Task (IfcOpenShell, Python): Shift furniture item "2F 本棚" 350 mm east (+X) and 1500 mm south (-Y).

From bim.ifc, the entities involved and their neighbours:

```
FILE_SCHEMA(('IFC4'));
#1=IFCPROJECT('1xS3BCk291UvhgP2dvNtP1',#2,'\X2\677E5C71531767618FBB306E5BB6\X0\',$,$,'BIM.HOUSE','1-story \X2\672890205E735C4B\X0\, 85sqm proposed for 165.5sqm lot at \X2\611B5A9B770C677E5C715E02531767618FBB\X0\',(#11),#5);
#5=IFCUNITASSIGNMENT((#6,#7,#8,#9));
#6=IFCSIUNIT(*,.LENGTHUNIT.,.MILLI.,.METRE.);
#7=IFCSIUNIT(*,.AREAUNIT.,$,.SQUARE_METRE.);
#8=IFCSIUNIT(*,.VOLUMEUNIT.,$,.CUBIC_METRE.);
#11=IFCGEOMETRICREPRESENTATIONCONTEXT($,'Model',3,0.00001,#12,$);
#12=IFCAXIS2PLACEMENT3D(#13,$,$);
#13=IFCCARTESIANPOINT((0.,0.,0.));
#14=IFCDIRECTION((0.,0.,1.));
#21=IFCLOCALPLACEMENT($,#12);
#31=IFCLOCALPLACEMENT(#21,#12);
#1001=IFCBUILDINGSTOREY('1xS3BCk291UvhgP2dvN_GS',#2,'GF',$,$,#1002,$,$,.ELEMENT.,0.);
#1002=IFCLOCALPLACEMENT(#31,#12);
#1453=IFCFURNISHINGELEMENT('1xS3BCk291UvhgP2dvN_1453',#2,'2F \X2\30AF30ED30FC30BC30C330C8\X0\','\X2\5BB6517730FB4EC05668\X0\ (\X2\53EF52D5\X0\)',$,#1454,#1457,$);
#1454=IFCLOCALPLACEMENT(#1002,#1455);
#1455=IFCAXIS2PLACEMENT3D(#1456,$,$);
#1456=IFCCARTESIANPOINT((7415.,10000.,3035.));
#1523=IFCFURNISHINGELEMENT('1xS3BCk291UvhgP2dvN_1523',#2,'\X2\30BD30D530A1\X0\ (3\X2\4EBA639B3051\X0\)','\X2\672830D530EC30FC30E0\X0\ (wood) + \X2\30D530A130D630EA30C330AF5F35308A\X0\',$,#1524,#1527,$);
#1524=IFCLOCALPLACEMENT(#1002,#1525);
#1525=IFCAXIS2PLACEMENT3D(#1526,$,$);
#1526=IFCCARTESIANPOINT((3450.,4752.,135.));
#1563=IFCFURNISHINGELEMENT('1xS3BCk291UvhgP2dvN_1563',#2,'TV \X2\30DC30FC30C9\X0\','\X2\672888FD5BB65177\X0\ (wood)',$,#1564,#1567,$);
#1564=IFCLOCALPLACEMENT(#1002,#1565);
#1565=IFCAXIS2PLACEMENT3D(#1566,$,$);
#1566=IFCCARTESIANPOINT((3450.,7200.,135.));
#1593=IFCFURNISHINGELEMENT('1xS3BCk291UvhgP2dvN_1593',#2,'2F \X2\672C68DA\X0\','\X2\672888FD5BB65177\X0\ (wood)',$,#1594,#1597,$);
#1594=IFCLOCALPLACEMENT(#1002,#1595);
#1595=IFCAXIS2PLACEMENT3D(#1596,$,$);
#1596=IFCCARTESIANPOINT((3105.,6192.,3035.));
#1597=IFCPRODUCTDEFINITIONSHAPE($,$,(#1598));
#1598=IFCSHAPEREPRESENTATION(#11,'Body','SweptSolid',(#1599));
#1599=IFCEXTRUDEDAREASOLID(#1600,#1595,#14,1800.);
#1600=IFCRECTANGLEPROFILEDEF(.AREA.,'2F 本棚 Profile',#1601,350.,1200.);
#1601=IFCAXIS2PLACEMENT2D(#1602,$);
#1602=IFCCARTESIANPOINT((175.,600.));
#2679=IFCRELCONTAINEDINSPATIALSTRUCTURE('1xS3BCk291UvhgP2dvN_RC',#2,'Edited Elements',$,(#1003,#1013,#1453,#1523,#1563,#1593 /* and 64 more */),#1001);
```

```python
import ifcopenshell
import ifcopenshell.api.geometry
import ifcopenshell.util.placement

model = ifcopenshell.open("bim.ifc")

item = model.by_guid("1xS3BCk291UvhgP2dvN_1593")
matrix = ifcopenshell.util.placement.get_local_placement(item.ObjectPlacement)
matrix[0, 3] += 350.0
matrix[1, 3] -= 1500.0
ifcopenshell.api.geometry.edit_object_placement(model, product=item, matrix=matrix, is_si=False)

print(ifcopenshell.util.placement.get_local_placement(item.ObjectPlacement).round(3) + 0.0)

model.write("bim-out.ifc")
```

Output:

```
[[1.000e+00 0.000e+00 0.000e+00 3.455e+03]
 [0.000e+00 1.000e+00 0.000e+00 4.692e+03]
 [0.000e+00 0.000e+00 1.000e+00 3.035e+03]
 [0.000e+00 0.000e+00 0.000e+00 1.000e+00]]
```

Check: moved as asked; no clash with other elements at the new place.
